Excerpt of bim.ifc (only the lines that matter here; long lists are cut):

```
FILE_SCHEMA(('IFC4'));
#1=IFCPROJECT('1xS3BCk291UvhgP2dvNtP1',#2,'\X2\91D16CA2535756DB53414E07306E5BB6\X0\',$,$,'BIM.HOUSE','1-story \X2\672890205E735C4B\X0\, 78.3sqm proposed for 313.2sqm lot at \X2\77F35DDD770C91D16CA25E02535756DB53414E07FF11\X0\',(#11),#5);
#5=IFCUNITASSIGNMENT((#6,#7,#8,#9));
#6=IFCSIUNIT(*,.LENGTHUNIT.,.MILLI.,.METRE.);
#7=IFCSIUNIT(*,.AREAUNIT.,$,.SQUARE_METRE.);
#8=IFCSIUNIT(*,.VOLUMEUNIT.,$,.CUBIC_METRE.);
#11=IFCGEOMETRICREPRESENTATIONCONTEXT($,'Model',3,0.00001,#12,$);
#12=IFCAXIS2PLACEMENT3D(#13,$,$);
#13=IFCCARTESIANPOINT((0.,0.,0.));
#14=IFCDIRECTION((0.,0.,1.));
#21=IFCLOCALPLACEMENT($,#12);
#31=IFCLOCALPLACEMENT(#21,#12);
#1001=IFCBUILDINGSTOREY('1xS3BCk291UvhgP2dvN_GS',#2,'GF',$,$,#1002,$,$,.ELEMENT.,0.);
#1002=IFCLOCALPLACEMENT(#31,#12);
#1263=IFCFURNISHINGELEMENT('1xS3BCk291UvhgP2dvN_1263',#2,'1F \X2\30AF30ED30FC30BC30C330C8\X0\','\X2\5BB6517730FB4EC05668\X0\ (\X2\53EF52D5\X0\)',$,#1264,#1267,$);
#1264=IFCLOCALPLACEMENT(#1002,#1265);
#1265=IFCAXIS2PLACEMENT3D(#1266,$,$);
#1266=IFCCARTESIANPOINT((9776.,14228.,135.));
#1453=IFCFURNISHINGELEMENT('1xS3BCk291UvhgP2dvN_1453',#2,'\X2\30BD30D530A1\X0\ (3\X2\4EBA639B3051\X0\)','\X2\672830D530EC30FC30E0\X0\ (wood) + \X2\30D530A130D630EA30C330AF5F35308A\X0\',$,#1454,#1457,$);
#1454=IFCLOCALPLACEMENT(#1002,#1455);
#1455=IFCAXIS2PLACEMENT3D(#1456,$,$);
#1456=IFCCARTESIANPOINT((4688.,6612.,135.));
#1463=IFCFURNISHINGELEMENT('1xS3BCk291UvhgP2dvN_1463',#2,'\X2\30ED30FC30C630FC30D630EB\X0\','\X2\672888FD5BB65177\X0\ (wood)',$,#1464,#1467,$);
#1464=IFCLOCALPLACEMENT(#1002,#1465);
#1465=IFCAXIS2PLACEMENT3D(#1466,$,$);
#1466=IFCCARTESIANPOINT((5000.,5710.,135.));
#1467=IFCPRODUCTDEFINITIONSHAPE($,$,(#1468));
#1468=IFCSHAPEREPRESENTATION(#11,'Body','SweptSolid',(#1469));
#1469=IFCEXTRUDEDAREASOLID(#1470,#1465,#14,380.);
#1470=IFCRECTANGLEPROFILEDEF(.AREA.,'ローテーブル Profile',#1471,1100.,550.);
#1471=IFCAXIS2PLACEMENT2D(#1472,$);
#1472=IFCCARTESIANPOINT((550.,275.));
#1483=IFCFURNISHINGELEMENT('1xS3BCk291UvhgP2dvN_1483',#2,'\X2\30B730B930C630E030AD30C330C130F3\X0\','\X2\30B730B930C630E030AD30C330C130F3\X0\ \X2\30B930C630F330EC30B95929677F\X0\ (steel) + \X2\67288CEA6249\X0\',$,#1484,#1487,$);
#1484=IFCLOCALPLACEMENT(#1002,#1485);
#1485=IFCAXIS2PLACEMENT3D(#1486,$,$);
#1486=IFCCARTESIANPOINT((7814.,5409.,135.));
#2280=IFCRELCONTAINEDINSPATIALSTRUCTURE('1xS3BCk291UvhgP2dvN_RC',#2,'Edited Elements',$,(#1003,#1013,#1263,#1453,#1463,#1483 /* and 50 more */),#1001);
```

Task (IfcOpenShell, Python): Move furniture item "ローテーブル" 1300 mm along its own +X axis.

```python
import ifcopenshell
import ifcopenshell.api.geometry
import ifcopenshell.util.placement
import ifcopenshell.util.unit

model = ifcopenshell.open("bim.ifc")
unit_scale = ifcopenshell.util.unit.calculate_unit_scale(model)

item = model.by_guid("1xS3BCk291UvhgP2dvN_1463")
matrix = ifcopenshell.util.placement.get_local_placement(item.ObjectPlacement)
matrix[:3, 3] += matrix[:3, 0] * 1.3 / unit_scale
ifcopenshell.api.geometry.edit_object_placement(model, product=item, matrix=matrix, is_si=False)

print(ifcopenshell.util.placement.get_local_placement(item.ObjectPlacement).round(3) + 0.0)

model.write("bim_rev.ifc")
```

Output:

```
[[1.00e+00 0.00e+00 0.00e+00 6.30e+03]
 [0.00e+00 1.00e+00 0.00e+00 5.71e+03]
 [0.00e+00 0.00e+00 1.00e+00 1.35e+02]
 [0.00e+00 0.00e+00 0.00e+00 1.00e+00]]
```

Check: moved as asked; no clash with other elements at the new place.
